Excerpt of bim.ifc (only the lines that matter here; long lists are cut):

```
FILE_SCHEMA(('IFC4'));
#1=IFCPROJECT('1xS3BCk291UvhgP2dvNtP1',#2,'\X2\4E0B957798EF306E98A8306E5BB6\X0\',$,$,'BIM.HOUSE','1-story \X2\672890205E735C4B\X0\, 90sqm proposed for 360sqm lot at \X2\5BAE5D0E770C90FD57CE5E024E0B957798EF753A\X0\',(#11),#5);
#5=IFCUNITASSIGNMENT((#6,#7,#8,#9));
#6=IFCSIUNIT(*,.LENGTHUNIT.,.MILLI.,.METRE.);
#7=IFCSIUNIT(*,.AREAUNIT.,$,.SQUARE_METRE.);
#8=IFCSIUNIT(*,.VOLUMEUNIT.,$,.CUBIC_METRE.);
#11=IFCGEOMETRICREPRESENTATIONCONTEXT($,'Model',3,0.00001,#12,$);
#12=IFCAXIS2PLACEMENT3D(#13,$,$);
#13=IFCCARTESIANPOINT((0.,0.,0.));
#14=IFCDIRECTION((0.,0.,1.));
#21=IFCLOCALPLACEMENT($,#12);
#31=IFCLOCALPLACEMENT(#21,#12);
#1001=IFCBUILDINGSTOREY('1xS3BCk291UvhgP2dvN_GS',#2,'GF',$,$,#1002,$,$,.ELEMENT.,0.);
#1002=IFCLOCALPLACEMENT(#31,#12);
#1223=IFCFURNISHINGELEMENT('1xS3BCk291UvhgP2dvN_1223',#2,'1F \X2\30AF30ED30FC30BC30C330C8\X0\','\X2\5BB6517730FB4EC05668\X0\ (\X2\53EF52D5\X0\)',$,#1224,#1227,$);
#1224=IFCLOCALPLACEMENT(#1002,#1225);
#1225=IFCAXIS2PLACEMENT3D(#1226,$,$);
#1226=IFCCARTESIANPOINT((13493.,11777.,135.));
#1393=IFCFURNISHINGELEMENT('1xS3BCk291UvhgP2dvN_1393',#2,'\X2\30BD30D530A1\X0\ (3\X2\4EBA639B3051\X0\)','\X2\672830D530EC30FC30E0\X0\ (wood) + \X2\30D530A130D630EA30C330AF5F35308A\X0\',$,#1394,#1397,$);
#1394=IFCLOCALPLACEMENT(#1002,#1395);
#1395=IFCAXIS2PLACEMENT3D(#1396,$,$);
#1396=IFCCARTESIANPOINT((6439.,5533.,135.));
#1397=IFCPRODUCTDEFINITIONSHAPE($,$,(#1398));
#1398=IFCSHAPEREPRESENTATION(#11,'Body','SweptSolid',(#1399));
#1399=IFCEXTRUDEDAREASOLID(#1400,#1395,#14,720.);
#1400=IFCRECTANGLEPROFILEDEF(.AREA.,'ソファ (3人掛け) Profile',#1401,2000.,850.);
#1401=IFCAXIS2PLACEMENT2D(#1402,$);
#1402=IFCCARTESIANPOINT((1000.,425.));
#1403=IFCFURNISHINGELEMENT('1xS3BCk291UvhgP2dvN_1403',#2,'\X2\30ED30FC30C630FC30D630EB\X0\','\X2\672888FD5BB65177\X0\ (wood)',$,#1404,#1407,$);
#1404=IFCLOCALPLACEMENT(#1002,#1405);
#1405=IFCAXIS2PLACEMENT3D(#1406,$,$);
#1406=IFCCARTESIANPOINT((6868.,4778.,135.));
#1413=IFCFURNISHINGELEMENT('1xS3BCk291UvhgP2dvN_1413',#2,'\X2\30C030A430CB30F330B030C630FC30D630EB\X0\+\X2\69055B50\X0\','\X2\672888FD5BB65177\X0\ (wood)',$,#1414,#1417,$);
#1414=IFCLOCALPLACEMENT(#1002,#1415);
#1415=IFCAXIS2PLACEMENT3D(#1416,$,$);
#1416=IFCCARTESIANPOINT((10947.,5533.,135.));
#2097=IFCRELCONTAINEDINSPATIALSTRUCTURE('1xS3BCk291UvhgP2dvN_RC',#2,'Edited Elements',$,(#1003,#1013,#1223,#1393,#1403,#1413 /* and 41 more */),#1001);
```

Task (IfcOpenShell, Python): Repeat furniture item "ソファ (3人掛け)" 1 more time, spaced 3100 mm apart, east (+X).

```python
import numpy as np
import ifcopenshell
import ifcopenshell.api.geometry
import ifcopenshell.api.root
import ifcopenshell.util.element
import ifcopenshell.util.placement
import ifcopenshell.util.unit

model = ifcopenshell.open("bim.ifc")
unit_scale = ifcopenshell.util.unit.calculate_unit_scale(model)


def reuse_history(source, copy):
    """copy_class also copies each property set's owner history, people and application; keep the originals."""
    for rel in copy.IsDefinedBy:
        if rel.is_a("IfcRelDefinesByProperties") and (history := rel.RelatingPropertyDefinition.OwnerHistory):
            rel.RelatingPropertyDefinition.OwnerHistory = source.OwnerHistory
            ifcopenshell.util.element.remove_deep2(model, history)


source = model.by_id(1393)
base = ifcopenshell.util.placement.get_local_placement(source.ObjectPlacement)
step = np.array([1.0, 0.0, 0.0]) * 3.1 / unit_scale

for i in range(1, 2):
    copy = ifcopenshell.api.root.copy_class(model, product=source)
    copy.Representation = ifcopenshell.util.element.copy_deep(
        model, source.Representation, exclude=["IfcGeometricRepresentationContext", "IfcRepresentationMap"]
    )
    reuse_history(source, copy)
    matrix = base.copy()
    matrix[:3, 3] += i * step
    print("added at", matrix[:3, 3].round(3) + 0.0)
    ifcopenshell.api.geometry.edit_object_placement(model, product=copy, matrix=matrix, is_si=False)

model.write("bim_edited.ifc")
```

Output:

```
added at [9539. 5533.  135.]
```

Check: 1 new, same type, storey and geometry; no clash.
